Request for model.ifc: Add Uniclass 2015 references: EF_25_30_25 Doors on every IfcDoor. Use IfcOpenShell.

First a look at what the model holds.

```python
import ifcopenshell

model = ifcopenshell.open("model.ifc")
print(model.schema)
print("classifications:", [c.Name for c in model.by_type("IfcClassification")])
for ifc_class in ("IfcDoor", "IfcRoof", "IfcStair", "IfcWall", "IfcWindow"):
    print(ifc_class, len(model.by_type(ifc_class)))
```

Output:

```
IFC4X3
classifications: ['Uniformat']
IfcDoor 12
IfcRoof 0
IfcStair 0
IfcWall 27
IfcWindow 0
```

```python
import ifcopenshell
import ifcopenshell.api.classification

model = ifcopenshell.open("model.ifc")

system = ifcopenshell.api.classification.add_classification(model, classification="Uniclass 2015")

codes = {
    "IfcDoor": ("EF_25_30_25", "Doors"),
}
for ifc_class, (code, name) in codes.items():
    products = model.by_type(ifc_class)
    ifcopenshell.api.classification.add_reference(
        model, products=products, classification=system, identification=code, name=name
    )
    print(code, len(products))

model.write("model-out.ifc")
```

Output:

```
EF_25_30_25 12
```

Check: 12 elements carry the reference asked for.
